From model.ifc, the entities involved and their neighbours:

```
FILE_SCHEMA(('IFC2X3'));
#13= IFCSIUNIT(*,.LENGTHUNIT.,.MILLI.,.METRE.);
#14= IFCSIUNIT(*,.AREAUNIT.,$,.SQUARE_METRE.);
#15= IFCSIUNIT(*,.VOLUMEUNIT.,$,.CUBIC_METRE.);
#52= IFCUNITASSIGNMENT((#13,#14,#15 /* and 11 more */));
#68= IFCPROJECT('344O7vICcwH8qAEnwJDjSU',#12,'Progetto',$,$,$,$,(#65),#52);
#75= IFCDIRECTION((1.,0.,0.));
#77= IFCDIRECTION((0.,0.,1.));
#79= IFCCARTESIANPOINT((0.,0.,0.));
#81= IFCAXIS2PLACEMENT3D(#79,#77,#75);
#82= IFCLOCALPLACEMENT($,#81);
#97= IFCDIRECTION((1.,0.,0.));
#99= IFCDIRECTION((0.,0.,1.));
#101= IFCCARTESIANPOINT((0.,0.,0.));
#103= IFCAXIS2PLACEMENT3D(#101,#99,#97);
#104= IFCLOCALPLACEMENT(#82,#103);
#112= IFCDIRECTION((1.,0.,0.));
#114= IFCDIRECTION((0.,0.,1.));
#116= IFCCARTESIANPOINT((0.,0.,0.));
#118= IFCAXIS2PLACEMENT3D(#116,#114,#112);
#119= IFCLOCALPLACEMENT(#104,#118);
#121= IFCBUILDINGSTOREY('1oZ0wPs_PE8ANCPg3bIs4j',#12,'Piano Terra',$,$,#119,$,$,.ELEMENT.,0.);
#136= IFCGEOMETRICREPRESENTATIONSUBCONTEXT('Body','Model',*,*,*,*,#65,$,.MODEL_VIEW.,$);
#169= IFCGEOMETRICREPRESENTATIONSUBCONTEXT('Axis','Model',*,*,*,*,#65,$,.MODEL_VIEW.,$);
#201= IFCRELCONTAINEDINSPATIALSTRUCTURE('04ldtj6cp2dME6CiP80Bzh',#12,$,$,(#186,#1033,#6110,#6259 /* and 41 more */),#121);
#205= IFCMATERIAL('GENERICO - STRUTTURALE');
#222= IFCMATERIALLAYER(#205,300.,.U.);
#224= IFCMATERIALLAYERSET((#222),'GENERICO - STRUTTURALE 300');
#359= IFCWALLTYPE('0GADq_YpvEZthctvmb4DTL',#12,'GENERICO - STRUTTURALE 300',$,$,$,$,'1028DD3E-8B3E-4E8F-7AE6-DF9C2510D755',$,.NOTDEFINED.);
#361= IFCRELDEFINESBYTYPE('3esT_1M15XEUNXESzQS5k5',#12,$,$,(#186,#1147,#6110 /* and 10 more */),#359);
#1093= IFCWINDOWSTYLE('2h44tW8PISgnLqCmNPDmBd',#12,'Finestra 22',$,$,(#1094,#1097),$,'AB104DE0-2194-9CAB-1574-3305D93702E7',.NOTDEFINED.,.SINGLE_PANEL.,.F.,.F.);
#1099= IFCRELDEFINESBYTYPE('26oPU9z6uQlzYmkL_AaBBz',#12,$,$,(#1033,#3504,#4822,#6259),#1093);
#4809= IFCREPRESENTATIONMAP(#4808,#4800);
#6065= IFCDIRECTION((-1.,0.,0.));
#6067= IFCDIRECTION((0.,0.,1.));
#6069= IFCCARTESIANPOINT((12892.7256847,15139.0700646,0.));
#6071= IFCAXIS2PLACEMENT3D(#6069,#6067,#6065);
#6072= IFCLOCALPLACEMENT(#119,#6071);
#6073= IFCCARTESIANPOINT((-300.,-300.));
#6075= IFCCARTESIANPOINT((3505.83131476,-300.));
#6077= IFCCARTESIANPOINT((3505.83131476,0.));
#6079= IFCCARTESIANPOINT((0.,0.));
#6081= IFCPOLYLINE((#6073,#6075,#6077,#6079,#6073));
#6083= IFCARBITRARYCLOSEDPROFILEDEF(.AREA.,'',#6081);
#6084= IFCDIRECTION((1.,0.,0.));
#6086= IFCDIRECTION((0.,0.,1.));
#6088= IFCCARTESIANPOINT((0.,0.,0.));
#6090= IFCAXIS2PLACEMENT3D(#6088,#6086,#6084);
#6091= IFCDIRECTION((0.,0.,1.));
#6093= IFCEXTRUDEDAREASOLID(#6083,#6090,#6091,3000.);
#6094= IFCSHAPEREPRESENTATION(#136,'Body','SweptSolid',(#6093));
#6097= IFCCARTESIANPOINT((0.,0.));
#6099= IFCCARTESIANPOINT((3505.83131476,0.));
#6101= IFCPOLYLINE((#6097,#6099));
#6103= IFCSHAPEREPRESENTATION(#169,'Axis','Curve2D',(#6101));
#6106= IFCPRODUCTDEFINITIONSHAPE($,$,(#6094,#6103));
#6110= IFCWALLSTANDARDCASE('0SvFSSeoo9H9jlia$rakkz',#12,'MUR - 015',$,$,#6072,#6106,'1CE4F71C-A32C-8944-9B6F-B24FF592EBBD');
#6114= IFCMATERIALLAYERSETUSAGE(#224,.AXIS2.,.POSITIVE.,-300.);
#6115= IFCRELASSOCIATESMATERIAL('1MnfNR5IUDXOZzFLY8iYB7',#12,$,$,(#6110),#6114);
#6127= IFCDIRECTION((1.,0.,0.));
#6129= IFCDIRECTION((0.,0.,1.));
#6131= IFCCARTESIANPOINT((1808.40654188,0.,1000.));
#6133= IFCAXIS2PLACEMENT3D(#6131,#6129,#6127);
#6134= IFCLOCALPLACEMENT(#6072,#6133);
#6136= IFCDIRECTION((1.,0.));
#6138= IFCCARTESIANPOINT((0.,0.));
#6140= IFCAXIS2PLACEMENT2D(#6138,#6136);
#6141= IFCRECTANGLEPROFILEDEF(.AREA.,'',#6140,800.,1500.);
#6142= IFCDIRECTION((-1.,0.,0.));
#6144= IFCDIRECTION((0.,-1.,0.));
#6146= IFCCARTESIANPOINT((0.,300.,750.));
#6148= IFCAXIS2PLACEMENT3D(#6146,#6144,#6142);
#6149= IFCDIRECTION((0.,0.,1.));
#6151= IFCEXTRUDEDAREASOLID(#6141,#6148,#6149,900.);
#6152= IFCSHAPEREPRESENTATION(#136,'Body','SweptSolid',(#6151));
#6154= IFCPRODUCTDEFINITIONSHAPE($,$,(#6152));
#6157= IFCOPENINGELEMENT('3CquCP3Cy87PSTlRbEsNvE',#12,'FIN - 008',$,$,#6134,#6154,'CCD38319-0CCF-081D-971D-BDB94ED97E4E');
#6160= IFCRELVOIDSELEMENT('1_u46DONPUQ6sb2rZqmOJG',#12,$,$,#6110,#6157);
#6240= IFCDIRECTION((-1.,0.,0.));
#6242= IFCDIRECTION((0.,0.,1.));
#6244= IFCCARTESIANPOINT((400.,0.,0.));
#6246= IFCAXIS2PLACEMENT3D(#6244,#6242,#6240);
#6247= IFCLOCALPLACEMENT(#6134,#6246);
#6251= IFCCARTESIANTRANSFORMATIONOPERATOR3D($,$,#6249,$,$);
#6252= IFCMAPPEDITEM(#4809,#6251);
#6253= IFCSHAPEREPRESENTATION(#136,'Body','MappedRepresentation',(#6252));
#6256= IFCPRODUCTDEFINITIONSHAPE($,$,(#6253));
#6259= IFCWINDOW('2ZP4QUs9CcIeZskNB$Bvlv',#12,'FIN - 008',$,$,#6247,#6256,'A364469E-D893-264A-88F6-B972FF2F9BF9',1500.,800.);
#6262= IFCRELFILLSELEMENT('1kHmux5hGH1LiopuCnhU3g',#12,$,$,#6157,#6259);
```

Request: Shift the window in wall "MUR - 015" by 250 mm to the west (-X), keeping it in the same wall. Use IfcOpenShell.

```python
import ifcopenshell
import ifcopenshell.api.geometry
import ifcopenshell.util.placement
import ifcopenshell.util.unit

model = ifcopenshell.open("model.ifc")
unit_scale = ifcopenshell.util.unit.calculate_unit_scale(model)

window = model.by_guid("2ZP4QUs9CcIeZskNB$Bvlv")
opening = window.FillsVoids[0].RelatingOpeningElement
wall = opening.VoidsElements[0].RelatingBuildingElement

wall_matrix = ifcopenshell.util.placement.get_local_placement(wall.ObjectPlacement)
shift = wall_matrix[:3, 0] * 0.25 / unit_scale
before = ifcopenshell.util.placement.get_local_placement(window.ObjectPlacement)[:3, 3].copy()

# The window is placed relative to its opening, so it follows when the opening moves.
matrix = ifcopenshell.util.placement.get_local_placement(opening.ObjectPlacement)
matrix[:3, 3] += shift
ifcopenshell.api.geometry.edit_object_placement(
    model, product=opening, matrix=matrix, is_si=False, should_transform_children=True
)

after = ifcopenshell.util.placement.get_local_placement(window.ObjectPlacement)[:3, 3]
print("window moved by", (after - before).round(3) + 0.0)

model.write("model-out.ifc")
```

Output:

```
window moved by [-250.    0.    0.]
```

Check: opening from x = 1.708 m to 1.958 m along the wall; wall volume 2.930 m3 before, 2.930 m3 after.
